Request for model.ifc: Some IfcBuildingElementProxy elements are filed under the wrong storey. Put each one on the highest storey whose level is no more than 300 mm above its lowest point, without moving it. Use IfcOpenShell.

First a look at what the model holds.

```python
import ifcopenshell
import ifcopenshell.util.element
import ifcopenshell.util.placement

model = ifcopenshell.open("model.ifc")
print(model.schema)
for storey in model.by_type("IfcBuildingStorey"):
    level = ifcopenshell.util.placement.get_storey_elevation(storey)
    count = sum(e.is_a("IfcBuildingElementProxy") for e in ifcopenshell.util.element.get_contained(storey))
    print(storey.id(), storey.Name, round(level, 3), count, sep=" | ")
```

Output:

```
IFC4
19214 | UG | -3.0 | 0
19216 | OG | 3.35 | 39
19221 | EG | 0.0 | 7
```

```python
import ifcopenshell
import ifcopenshell.api.spatial
import ifcopenshell.geom
import ifcopenshell.util.element
import ifcopenshell.util.placement
import ifcopenshell.util.shape
import ifcopenshell.util.unit

model = ifcopenshell.open("model.ifc")
unit_scale = ifcopenshell.util.unit.calculate_unit_scale(model)
settings = ifcopenshell.geom.settings()

levels = sorted(
    ((ifcopenshell.util.placement.get_storey_elevation(s) * unit_scale, s) for s in model.by_type("IfcBuildingStorey")),
    key=lambda pair: pair[0],
)

for e in model.by_type("IfcBuildingElementProxy"):
    current = e.ContainedInStructure[0].RelatingStructure if e.ContainedInStructure else None
    if current is None or not current.is_a("IfcBuildingStorey"):
        continue
    shape = ifcopenshell.geom.create_shape(settings, e)
    bottom = ifcopenshell.util.shape.get_shape_bottom_elevation(shape, shape.geometry)
    below = [s for level, s in levels if level <= bottom + 0.3]
    storey = below[-1] if below else levels[0][1]
    if storey != current:
        # assign_container keeps the world position.
        ifcopenshell.api.spatial.assign_container(model, products=[e], relating_structure=storey)
        print(e.id(), current.Name, "->", storey.Name)

model.write("model_v2.ifc")
```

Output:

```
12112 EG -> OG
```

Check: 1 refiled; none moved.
